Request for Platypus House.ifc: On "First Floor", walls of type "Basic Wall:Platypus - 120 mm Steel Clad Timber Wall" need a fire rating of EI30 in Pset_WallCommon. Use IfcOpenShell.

First a look at what the model holds.

```python
import ifcopenshell
import ifcopenshell.util.element

model = ifcopenshell.open("Platypus House.ifc")
print(model.schema)
storey = next(s for s in model.by_type("IfcBuildingStorey") if s.Name == "First Floor")
walls = [e for e in ifcopenshell.util.element.get_decomposition(storey) if e.is_a("IfcWall")]
seen = {}
for e in walls:
    element_type = ifcopenshell.util.element.get_type(e)
    key = (element_type.Name if element_type != e and element_type else None, ifcopenshell.util.element.get_pset(e, "Pset_WallCommon", "FireRating"))
    seen[key] = seen.get(key, 0) + 1
for (name, value), count in sorted(seen.items(), key=str):
    print(count, "x", name, "|", value)
```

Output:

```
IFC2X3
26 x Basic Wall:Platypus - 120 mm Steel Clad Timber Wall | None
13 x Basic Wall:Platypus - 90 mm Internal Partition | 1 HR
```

```python
import ifcopenshell
import ifcopenshell.api.pset
import ifcopenshell.util.element

model = ifcopenshell.open("Platypus House.ifc")

storey = next(s for s in model.by_type("IfcBuildingStorey") if s.Name == "First Floor")
walls = [e for e in ifcopenshell.util.element.get_decomposition(storey) if e.is_a("IfcWall")]

count = 0
for e in walls:
    element_type = ifcopenshell.util.element.get_type(e)
    if element_type in (None, e) or element_type.Name != "Basic Wall:Platypus - 120 mm Steel Clad Timber Wall":
        continue
    # add_pset returns the element's existing set when there is one.
    pset = ifcopenshell.api.pset.add_pset(model, product=e, name="Pset_WallCommon")
    ifcopenshell.api.pset.edit_pset(model, pset=pset, properties={"FireRating": "EI30"})
    count += 1

print(count, "walls updated")

model.write("Platypus House-out.ifc")
```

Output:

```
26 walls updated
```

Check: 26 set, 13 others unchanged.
